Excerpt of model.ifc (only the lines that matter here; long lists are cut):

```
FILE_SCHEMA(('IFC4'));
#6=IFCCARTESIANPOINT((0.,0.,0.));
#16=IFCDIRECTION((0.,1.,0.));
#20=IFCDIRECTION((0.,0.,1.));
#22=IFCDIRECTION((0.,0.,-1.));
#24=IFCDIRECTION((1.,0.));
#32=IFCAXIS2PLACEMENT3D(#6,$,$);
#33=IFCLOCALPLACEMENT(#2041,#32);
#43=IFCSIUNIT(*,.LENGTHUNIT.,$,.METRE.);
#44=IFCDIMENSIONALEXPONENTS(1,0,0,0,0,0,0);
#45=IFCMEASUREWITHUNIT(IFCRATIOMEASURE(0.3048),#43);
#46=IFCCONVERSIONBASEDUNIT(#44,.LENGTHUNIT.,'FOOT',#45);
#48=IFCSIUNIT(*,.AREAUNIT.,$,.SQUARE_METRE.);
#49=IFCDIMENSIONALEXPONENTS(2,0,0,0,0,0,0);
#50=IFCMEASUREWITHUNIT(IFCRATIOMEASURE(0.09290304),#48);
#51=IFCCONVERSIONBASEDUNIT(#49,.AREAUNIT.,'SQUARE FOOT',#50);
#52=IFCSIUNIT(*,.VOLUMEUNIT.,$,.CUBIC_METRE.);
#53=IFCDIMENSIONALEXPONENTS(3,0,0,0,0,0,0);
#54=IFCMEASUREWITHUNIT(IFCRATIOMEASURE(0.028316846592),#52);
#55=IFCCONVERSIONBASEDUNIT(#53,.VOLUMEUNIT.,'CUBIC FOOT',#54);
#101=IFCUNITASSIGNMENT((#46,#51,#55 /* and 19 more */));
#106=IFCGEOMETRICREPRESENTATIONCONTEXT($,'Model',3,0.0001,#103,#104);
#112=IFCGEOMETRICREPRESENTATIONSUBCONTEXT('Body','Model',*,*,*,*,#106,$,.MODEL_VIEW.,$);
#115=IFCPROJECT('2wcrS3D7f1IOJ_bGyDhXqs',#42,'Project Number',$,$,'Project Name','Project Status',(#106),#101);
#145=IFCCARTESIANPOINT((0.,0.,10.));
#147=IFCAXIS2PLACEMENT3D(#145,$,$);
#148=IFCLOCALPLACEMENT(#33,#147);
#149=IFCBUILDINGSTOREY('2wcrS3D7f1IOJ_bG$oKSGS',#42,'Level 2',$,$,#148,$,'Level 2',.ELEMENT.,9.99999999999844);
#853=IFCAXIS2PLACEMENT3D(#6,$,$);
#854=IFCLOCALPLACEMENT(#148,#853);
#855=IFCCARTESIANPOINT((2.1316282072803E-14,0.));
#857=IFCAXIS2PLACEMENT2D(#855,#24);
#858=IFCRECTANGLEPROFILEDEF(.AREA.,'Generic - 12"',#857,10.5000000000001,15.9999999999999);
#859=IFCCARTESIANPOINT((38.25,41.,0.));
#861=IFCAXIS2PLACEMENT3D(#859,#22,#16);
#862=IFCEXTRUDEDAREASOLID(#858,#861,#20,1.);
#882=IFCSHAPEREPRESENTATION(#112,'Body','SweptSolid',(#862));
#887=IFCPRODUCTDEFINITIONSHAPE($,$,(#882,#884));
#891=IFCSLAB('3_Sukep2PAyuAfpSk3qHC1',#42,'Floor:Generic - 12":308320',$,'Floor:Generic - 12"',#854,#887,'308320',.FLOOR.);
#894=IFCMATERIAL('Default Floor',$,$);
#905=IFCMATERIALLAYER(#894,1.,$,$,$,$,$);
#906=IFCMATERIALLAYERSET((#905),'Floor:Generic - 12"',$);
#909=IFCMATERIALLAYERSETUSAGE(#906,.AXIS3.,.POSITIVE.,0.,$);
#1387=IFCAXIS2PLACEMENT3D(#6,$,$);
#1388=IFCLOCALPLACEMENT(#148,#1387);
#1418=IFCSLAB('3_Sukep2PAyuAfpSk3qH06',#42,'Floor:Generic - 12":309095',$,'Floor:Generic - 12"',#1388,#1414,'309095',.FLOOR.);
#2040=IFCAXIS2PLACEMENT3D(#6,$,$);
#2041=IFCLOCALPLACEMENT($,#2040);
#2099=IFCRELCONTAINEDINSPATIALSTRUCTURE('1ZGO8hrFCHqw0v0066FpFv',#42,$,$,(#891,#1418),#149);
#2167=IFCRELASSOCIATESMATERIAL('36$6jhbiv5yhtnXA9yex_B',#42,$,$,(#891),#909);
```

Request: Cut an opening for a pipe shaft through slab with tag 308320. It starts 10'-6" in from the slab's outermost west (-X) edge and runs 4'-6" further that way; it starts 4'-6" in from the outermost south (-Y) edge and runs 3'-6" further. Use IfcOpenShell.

```python
import numpy as np
import ifcopenshell
import ifcopenshell.api.feature
import ifcopenshell.api.geometry
import ifcopenshell.api.root
import ifcopenshell.geom
import ifcopenshell.util.placement
import ifcopenshell.util.representation
import ifcopenshell.util.shape
import ifcopenshell.util.unit

model = ifcopenshell.open("model.ifc")
unit_scale = ifcopenshell.util.unit.calculate_unit_scale(model)
settings = ifcopenshell.geom.settings()


def volume(element):
    """Net volume in cubic metres, openings subtracted."""
    shape = ifcopenshell.geom.create_shape(settings, element)
    return ifcopenshell.util.shape.get_volume(shape.geometry)


slab = model.by_id(891)
before = volume(slab)

# Extent in the slab's own axes, in metres. The edges named are its -X and -Y sides.
slab_shape = ifcopenshell.geom.create_shape(settings, slab)
vertices = ifcopenshell.util.shape.get_vertices(slab_shape.geometry)
x_min, y_min, bottom = vertices.min(axis=0)
top = vertices[:, 2].max()

opening = ifcopenshell.api.root.create_entity(model, ifc_class="IfcOpeningElement", name="Pipe shaft opening", predefined_type="OPENING")
context = ifcopenshell.util.representation.get_context(model, "Model", "Body", "MODEL_VIEW")
width, depth = 1.3716, 1.0668
outline = [(0.0, 0.0), (width, 0.0), (width, depth), (0.0, depth), (0.0, 0.0)]
# Overshoot both faces by 50 mm so the cut is clean.
shape = ifcopenshell.api.geometry.add_slab_representation(
    model, context=context, depth=top - bottom + 0.1, polyline=outline
)
ifcopenshell.api.geometry.assign_representation(model, product=opening, representation=shape)

matrix = ifcopenshell.util.placement.get_local_placement(slab.ObjectPlacement)
matrix[:, 3] = matrix @ np.append(np.array([x_min + 3.2004, y_min + 1.3716, bottom - 0.05]) / unit_scale, 1.0)
ifcopenshell.api.geometry.edit_object_placement(model, product=opening, matrix=matrix, is_si=False)
ifcopenshell.api.feature.add_feature(model, feature=opening, element=slab)

after = volume(slab)

print(f"slab volume {before:.3f} -> {after:.3f} m3")

model.write("model_rev.ifc")
```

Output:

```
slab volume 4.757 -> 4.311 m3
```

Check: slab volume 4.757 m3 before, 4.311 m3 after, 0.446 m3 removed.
